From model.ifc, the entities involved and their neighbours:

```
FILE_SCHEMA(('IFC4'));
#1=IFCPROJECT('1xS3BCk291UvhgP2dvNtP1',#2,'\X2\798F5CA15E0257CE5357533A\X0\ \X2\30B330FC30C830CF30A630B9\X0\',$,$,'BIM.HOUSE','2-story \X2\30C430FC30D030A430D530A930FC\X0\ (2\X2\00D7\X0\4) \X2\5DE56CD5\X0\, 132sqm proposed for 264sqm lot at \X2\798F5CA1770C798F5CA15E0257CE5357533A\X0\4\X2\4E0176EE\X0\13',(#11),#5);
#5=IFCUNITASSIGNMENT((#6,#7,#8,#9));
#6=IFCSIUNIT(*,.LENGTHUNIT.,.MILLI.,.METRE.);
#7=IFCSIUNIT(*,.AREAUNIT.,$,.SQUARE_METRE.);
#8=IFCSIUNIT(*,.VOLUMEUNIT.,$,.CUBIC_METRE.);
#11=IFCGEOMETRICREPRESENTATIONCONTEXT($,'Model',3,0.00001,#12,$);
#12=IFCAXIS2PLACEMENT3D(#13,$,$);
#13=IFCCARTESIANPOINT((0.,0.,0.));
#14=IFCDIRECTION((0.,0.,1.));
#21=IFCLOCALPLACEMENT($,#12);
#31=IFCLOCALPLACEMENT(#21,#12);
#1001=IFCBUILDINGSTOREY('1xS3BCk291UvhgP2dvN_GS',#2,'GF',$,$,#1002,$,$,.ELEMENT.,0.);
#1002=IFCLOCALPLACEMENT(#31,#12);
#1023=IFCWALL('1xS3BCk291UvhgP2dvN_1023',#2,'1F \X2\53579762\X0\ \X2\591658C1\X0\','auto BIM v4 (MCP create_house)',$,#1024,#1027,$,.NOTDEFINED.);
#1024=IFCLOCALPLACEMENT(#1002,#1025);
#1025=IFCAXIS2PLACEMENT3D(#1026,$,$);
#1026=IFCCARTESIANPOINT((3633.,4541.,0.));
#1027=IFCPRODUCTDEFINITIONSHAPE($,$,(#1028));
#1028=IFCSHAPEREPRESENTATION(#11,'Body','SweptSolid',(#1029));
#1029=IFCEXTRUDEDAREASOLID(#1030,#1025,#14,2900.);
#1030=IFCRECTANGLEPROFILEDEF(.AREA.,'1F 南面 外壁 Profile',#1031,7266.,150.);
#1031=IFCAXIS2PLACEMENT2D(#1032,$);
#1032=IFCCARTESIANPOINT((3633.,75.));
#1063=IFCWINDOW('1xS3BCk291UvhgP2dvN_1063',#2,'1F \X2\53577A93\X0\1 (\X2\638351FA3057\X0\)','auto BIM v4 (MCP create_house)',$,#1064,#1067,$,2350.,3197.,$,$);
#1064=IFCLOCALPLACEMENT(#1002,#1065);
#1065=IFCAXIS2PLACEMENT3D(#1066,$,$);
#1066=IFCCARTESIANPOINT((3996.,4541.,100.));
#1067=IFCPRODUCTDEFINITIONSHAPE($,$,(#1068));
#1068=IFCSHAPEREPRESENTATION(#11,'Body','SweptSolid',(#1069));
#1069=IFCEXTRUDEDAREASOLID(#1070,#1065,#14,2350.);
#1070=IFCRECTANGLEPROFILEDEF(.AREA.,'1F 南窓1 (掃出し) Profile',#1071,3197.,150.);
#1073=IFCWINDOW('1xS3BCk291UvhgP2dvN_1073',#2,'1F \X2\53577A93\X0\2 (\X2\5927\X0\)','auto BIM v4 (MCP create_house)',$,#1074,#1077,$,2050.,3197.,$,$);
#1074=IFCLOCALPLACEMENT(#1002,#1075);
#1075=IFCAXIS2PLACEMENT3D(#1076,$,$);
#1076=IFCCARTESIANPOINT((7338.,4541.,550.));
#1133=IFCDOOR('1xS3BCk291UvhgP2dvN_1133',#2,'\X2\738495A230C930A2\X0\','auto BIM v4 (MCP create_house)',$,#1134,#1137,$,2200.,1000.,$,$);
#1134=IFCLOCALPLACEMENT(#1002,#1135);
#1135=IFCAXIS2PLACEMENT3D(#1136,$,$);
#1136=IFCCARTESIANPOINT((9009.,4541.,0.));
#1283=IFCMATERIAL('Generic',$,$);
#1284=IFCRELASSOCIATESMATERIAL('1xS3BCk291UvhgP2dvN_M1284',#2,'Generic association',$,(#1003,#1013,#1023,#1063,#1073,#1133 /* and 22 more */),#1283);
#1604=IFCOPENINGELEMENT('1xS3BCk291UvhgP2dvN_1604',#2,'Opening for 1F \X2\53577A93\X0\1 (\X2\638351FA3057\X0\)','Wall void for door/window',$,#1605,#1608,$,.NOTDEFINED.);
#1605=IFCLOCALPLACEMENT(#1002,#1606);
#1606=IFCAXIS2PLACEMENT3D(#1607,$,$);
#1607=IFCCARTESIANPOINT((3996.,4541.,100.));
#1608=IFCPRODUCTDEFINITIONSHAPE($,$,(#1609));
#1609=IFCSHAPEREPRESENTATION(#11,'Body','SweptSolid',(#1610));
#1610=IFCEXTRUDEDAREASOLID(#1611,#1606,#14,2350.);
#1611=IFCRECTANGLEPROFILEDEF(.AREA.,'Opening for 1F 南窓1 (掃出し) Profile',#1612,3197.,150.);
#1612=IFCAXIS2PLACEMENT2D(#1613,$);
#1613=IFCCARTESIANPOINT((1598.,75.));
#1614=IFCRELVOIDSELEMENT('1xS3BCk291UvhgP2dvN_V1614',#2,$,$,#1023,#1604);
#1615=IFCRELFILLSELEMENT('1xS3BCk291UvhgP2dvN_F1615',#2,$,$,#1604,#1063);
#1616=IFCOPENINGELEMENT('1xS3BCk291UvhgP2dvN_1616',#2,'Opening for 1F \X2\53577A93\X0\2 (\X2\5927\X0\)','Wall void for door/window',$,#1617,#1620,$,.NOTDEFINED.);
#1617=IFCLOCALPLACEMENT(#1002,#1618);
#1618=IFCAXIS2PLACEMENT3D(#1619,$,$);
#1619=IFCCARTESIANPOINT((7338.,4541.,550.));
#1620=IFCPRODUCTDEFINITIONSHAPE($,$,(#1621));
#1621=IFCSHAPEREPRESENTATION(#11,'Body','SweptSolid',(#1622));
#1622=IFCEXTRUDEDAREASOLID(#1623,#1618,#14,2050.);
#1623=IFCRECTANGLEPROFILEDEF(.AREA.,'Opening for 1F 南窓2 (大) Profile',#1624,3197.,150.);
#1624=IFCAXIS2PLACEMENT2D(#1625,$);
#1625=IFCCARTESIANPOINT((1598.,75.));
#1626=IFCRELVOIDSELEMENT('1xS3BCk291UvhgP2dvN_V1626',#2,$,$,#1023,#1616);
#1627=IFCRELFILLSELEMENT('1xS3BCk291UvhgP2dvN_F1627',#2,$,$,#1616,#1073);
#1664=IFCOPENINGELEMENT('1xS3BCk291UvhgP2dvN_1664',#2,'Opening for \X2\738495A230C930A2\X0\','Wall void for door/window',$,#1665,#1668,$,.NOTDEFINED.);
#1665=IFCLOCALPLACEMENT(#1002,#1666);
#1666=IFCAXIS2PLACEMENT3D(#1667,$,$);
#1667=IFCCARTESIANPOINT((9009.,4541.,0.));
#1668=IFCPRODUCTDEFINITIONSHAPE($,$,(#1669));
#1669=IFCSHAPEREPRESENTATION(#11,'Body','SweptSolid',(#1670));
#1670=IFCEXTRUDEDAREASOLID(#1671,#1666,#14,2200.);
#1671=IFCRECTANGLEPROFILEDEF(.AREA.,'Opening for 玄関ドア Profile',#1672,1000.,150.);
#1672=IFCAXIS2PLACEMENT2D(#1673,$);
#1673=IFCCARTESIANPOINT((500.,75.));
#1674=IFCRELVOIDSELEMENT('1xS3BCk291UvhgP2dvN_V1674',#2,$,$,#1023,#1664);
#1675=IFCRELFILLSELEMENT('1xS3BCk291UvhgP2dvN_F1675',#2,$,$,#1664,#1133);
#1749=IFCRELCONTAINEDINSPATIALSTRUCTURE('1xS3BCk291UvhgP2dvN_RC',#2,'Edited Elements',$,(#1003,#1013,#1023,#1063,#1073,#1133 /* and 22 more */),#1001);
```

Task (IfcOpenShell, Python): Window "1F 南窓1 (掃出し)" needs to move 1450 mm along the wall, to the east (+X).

```python
import ifcopenshell
import ifcopenshell.api.geometry
import ifcopenshell.util.placement
import ifcopenshell.util.unit

model = ifcopenshell.open("model.ifc")
unit_scale = ifcopenshell.util.unit.calculate_unit_scale(model)

window = model.by_id(1063)
opening = window.FillsVoids[0].RelatingOpeningElement
wall = opening.VoidsElements[0].RelatingBuildingElement

wall_matrix = ifcopenshell.util.placement.get_local_placement(wall.ObjectPlacement)
shift = wall_matrix[:3, 0] * 1.45 / unit_scale
before = ifcopenshell.util.placement.get_local_placement(window.ObjectPlacement)[:3, 3].copy()

# The window is not placed relative to its opening, so move both.
for product in (opening, window):
    matrix = ifcopenshell.util.placement.get_local_placement(product.ObjectPlacement)
    matrix[:3, 3] += shift
    ifcopenshell.api.geometry.edit_object_placement(model, product=product, matrix=matrix, is_si=False)

after = ifcopenshell.util.placement.get_local_placement(window.ObjectPlacement)[:3, 3]
print("window moved by", (after - before).round(3) + 0.0)

model.write("model-out.ifc")
```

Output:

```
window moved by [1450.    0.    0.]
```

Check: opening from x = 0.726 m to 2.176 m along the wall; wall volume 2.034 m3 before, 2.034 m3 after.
